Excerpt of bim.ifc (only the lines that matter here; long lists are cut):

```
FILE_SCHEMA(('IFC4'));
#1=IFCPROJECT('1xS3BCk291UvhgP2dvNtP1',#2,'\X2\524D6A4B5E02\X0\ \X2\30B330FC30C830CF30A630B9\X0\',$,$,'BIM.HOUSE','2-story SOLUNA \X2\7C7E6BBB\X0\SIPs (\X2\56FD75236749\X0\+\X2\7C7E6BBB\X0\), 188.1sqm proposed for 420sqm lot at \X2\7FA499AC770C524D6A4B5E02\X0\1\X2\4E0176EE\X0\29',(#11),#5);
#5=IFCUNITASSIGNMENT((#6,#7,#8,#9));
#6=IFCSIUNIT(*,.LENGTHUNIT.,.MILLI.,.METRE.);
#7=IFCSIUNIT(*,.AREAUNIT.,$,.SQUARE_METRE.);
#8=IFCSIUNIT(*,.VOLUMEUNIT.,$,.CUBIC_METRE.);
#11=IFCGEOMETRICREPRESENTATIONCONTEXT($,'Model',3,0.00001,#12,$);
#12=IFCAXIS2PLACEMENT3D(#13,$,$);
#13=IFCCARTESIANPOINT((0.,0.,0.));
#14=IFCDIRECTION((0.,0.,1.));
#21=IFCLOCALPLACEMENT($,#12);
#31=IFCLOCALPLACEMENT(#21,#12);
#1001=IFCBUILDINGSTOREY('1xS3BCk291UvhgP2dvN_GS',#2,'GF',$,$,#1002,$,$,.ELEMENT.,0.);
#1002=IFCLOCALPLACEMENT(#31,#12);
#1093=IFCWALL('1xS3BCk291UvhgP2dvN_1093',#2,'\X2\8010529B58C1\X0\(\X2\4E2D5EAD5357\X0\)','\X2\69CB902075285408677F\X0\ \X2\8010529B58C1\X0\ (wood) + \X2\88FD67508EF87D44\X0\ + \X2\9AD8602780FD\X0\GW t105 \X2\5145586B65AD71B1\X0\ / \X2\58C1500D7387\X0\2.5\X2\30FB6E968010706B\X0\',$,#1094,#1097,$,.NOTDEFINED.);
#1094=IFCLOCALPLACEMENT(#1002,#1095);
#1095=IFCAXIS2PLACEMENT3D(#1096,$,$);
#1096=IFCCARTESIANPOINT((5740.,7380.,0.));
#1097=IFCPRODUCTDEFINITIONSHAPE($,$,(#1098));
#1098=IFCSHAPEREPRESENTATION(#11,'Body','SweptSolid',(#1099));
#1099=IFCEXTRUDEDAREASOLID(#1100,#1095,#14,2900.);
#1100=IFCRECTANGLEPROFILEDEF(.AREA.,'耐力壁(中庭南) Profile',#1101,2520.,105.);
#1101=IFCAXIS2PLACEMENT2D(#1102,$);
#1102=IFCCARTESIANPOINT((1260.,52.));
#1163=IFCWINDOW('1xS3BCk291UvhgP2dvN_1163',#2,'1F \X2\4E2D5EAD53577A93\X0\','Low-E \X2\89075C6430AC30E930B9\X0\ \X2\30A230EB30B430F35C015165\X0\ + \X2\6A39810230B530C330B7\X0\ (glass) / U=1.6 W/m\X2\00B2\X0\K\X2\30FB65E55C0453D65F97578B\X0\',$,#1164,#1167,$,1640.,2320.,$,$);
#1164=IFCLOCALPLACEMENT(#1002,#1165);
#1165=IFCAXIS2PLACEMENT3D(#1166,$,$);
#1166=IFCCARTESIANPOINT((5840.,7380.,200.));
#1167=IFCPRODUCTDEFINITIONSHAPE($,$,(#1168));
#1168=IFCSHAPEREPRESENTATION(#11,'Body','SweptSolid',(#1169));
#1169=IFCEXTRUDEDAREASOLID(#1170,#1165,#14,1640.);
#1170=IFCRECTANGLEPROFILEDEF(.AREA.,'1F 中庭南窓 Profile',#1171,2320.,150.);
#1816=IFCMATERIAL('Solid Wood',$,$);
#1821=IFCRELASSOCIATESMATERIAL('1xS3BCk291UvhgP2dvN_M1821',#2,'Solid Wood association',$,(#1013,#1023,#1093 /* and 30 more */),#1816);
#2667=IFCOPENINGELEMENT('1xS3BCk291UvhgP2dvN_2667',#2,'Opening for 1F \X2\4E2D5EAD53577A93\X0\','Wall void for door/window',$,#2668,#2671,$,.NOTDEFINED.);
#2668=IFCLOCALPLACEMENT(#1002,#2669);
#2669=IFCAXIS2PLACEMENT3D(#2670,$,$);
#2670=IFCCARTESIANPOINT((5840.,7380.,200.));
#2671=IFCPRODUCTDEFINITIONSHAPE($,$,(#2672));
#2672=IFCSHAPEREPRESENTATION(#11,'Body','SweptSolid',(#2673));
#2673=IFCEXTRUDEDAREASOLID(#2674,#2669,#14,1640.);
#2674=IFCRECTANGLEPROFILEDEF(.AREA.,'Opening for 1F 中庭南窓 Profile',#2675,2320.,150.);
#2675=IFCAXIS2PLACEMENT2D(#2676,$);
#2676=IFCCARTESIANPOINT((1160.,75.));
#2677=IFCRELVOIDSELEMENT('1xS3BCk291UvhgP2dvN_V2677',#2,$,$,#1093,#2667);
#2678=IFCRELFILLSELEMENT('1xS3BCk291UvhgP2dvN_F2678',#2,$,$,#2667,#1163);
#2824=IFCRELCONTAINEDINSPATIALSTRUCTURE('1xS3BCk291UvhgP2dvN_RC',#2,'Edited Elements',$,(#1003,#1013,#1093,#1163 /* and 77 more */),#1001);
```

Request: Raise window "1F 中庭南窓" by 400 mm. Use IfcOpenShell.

```python
import numpy as np
import ifcopenshell
import ifcopenshell.api.geometry
import ifcopenshell.util.placement
import ifcopenshell.util.unit

model = ifcopenshell.open("bim.ifc")
unit_scale = ifcopenshell.util.unit.calculate_unit_scale(model)

window = model.by_guid("1xS3BCk291UvhgP2dvN_1163")
opening = window.FillsVoids[0].RelatingOpeningElement
dz = 0.4 / unit_scale

shift = np.array([0.0, 0.0, dz])
# The window is not placed relative to its opening, so move both.
for product in (opening, window):
    matrix = ifcopenshell.util.placement.get_local_placement(product.ObjectPlacement)
    matrix[:3, 3] += shift
    ifcopenshell.api.geometry.edit_object_placement(model, product=product, matrix=matrix, is_si=False)

print(f"moved by {dz * unit_scale:+.3f} m")

model.write("bim_updated.ifc")
```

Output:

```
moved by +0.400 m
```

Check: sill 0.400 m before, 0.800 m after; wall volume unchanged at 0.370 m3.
